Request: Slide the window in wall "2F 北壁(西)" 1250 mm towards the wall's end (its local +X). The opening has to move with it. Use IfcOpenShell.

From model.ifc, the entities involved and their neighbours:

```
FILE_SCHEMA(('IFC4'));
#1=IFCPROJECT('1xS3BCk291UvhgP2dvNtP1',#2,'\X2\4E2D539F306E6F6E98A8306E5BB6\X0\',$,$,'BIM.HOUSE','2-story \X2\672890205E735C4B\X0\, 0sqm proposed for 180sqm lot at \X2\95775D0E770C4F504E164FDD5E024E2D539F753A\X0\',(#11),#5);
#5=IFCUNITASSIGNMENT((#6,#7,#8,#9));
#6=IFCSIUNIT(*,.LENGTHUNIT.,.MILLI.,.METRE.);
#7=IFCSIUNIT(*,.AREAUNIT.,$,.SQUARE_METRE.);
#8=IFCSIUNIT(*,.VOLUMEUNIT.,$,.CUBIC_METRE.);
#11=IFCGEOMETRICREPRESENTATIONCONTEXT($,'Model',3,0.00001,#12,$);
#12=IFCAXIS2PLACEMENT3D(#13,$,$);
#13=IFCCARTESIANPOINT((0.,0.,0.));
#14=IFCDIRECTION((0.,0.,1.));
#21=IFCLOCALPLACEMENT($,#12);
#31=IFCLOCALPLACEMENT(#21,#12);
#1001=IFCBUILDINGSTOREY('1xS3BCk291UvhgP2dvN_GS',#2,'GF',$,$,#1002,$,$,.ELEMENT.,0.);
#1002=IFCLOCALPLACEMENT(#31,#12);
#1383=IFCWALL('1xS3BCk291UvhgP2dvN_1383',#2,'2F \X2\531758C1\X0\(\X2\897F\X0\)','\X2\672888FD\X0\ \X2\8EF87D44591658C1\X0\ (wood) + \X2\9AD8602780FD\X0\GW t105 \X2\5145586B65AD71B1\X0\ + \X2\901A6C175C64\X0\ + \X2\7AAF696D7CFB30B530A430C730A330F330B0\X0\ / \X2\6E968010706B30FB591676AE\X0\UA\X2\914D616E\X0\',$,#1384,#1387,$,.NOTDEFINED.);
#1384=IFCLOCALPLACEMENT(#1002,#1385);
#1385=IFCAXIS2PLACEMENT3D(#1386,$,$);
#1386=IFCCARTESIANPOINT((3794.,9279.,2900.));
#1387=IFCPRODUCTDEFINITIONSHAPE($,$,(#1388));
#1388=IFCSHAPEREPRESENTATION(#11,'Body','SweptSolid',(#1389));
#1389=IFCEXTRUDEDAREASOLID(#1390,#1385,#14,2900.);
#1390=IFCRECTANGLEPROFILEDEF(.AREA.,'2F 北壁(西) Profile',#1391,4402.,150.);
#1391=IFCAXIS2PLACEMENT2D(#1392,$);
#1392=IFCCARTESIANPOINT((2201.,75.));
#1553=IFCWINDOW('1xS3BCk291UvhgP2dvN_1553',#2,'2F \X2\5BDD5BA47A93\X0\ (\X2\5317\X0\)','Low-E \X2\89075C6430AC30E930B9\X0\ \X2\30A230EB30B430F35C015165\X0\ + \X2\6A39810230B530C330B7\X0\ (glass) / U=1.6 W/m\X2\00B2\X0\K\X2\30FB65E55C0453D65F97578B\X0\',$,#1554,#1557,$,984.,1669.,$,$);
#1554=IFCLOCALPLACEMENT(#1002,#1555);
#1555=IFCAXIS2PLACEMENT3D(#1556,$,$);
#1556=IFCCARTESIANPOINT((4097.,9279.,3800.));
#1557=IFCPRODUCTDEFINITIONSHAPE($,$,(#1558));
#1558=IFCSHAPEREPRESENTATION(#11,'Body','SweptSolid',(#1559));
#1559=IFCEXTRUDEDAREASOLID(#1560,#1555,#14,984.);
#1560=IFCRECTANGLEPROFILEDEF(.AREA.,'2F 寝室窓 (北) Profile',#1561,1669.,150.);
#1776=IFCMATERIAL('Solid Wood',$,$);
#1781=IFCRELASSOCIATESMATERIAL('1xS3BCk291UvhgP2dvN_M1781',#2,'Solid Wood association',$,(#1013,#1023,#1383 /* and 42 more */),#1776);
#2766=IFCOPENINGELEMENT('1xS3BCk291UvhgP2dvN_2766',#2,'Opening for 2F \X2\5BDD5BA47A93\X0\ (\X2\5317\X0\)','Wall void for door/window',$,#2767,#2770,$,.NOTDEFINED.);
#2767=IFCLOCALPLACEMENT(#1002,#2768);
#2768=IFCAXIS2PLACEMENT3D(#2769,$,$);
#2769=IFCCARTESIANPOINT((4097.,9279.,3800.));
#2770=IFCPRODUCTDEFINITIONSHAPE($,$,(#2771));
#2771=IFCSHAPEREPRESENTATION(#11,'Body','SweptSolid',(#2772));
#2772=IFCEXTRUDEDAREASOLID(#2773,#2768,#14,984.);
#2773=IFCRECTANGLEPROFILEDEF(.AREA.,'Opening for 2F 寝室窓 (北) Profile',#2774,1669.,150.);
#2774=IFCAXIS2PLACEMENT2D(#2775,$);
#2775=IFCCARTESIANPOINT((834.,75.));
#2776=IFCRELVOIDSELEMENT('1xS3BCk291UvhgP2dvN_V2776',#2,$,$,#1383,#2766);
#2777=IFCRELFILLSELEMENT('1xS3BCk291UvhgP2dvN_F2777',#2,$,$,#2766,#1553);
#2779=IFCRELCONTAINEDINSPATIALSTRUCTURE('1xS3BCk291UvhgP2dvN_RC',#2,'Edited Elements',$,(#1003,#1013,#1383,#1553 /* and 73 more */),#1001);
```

```python
import ifcopenshell
import ifcopenshell.api.geometry
import ifcopenshell.util.placement

model = ifcopenshell.open("model.ifc")

window = model.by_id(1553)
opening = window.FillsVoids[0].RelatingOpeningElement
wall = opening.VoidsElements[0].RelatingBuildingElement

wall_matrix = ifcopenshell.util.placement.get_local_placement(wall.ObjectPlacement)
shift = wall_matrix[:3, 0] * 1250.0
before = ifcopenshell.util.placement.get_local_placement(window.ObjectPlacement)[:3, 3].copy()

# The window is not placed relative to its opening, so move both.
for product in (opening, window):
    matrix = ifcopenshell.util.placement.get_local_placement(product.ObjectPlacement)
    matrix[:3, 3] += shift
    ifcopenshell.api.geometry.edit_object_placement(model, product=product, matrix=matrix, is_si=False)

after = ifcopenshell.util.placement.get_local_placement(window.ObjectPlacement)[:3, 3]
print("window moved by", (after - before).round(3) + 0.0)

model.write("model_updated.ifc")
```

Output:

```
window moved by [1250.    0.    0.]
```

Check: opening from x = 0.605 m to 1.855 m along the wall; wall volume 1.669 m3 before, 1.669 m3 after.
